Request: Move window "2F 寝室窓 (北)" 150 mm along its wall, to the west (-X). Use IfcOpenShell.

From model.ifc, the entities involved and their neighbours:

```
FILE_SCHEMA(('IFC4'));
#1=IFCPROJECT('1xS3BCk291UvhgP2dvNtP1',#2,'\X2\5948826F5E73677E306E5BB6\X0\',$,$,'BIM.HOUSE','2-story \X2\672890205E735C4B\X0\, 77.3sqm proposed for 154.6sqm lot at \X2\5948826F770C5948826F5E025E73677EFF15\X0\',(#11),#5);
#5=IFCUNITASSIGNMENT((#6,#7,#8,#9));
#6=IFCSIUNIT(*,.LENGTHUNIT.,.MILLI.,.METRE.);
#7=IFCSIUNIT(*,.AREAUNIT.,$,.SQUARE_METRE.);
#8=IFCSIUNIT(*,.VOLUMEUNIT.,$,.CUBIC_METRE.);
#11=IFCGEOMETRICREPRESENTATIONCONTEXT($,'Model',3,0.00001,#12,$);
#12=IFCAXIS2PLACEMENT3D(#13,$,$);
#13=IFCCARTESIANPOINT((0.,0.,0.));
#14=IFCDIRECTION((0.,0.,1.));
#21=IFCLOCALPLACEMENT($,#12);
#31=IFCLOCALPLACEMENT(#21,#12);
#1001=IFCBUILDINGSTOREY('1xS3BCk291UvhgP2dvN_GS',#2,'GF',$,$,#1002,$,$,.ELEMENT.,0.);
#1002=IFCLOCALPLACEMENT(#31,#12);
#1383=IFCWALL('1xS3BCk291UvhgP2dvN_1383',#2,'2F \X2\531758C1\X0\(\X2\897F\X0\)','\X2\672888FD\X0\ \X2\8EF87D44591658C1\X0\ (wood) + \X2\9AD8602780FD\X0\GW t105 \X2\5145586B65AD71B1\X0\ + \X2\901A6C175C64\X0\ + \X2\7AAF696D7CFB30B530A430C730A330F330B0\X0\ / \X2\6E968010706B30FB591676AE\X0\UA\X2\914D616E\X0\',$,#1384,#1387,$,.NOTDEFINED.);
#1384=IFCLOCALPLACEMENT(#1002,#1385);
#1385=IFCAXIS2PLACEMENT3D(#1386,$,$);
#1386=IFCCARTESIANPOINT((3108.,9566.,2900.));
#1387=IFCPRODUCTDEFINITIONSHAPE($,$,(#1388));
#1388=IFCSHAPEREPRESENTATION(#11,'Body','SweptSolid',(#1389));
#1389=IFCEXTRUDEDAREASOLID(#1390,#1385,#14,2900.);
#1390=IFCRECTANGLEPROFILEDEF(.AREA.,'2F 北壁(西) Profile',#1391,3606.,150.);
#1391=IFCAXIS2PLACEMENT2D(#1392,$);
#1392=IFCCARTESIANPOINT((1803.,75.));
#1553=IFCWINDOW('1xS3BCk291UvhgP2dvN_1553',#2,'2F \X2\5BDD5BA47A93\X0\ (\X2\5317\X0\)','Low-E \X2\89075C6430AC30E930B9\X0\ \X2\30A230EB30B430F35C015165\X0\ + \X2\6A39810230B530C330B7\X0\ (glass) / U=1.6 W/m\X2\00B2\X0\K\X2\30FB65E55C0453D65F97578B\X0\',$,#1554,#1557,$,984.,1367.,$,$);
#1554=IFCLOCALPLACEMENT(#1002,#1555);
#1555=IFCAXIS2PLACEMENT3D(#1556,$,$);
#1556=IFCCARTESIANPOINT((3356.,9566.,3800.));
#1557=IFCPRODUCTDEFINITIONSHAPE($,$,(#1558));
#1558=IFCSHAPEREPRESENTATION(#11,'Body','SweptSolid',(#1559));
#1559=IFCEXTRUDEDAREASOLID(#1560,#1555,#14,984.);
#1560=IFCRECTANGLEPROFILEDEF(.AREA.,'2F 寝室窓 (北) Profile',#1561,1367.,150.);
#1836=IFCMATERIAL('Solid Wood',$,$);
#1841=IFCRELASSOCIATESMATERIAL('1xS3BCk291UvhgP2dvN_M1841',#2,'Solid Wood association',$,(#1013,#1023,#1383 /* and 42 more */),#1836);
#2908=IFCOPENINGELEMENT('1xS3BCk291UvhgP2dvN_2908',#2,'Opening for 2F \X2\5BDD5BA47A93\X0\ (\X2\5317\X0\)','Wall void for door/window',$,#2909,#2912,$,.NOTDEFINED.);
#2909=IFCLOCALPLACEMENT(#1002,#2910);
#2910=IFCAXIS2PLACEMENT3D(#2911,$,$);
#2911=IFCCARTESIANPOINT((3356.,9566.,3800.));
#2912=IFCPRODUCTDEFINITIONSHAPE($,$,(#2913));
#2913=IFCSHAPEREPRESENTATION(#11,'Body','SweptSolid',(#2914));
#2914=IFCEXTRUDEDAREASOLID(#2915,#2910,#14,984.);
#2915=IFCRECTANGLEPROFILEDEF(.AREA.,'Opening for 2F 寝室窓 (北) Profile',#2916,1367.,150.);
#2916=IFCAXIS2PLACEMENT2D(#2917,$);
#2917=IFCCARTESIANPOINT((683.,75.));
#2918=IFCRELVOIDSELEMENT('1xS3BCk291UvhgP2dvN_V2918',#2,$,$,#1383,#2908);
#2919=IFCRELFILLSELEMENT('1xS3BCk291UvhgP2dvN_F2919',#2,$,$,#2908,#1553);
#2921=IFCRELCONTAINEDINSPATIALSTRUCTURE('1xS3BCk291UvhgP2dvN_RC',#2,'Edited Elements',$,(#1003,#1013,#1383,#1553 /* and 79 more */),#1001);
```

```python
import ifcopenshell
import ifcopenshell.api.geometry
import ifcopenshell.util.placement

model = ifcopenshell.open("model.ifc")

window = model.by_guid("1xS3BCk291UvhgP2dvN_1553")
opening = window.FillsVoids[0].RelatingOpeningElement
wall = opening.VoidsElements[0].RelatingBuildingElement

wall_matrix = ifcopenshell.util.placement.get_local_placement(wall.ObjectPlacement)
shift = wall_matrix[:3, 0] * -150.0
before = ifcopenshell.util.placement.get_local_placement(window.ObjectPlacement)[:3, 3].copy()

# The window is not placed relative to its opening, so move both.
for product in (opening, window):
    matrix = ifcopenshell.util.placement.get_local_placement(product.ObjectPlacement)
    matrix[:3, 3] += shift
    ifcopenshell.api.geometry.edit_object_placement(model, product=product, matrix=matrix, is_si=False)

after = ifcopenshell.util.placement.get_local_placement(window.ObjectPlacement)[:3, 3]
print("window moved by", (after - before).round(3) + 0.0)

model.write("model_updated.ifc")
```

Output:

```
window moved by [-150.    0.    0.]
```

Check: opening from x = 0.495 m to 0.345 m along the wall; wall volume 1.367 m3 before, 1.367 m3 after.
